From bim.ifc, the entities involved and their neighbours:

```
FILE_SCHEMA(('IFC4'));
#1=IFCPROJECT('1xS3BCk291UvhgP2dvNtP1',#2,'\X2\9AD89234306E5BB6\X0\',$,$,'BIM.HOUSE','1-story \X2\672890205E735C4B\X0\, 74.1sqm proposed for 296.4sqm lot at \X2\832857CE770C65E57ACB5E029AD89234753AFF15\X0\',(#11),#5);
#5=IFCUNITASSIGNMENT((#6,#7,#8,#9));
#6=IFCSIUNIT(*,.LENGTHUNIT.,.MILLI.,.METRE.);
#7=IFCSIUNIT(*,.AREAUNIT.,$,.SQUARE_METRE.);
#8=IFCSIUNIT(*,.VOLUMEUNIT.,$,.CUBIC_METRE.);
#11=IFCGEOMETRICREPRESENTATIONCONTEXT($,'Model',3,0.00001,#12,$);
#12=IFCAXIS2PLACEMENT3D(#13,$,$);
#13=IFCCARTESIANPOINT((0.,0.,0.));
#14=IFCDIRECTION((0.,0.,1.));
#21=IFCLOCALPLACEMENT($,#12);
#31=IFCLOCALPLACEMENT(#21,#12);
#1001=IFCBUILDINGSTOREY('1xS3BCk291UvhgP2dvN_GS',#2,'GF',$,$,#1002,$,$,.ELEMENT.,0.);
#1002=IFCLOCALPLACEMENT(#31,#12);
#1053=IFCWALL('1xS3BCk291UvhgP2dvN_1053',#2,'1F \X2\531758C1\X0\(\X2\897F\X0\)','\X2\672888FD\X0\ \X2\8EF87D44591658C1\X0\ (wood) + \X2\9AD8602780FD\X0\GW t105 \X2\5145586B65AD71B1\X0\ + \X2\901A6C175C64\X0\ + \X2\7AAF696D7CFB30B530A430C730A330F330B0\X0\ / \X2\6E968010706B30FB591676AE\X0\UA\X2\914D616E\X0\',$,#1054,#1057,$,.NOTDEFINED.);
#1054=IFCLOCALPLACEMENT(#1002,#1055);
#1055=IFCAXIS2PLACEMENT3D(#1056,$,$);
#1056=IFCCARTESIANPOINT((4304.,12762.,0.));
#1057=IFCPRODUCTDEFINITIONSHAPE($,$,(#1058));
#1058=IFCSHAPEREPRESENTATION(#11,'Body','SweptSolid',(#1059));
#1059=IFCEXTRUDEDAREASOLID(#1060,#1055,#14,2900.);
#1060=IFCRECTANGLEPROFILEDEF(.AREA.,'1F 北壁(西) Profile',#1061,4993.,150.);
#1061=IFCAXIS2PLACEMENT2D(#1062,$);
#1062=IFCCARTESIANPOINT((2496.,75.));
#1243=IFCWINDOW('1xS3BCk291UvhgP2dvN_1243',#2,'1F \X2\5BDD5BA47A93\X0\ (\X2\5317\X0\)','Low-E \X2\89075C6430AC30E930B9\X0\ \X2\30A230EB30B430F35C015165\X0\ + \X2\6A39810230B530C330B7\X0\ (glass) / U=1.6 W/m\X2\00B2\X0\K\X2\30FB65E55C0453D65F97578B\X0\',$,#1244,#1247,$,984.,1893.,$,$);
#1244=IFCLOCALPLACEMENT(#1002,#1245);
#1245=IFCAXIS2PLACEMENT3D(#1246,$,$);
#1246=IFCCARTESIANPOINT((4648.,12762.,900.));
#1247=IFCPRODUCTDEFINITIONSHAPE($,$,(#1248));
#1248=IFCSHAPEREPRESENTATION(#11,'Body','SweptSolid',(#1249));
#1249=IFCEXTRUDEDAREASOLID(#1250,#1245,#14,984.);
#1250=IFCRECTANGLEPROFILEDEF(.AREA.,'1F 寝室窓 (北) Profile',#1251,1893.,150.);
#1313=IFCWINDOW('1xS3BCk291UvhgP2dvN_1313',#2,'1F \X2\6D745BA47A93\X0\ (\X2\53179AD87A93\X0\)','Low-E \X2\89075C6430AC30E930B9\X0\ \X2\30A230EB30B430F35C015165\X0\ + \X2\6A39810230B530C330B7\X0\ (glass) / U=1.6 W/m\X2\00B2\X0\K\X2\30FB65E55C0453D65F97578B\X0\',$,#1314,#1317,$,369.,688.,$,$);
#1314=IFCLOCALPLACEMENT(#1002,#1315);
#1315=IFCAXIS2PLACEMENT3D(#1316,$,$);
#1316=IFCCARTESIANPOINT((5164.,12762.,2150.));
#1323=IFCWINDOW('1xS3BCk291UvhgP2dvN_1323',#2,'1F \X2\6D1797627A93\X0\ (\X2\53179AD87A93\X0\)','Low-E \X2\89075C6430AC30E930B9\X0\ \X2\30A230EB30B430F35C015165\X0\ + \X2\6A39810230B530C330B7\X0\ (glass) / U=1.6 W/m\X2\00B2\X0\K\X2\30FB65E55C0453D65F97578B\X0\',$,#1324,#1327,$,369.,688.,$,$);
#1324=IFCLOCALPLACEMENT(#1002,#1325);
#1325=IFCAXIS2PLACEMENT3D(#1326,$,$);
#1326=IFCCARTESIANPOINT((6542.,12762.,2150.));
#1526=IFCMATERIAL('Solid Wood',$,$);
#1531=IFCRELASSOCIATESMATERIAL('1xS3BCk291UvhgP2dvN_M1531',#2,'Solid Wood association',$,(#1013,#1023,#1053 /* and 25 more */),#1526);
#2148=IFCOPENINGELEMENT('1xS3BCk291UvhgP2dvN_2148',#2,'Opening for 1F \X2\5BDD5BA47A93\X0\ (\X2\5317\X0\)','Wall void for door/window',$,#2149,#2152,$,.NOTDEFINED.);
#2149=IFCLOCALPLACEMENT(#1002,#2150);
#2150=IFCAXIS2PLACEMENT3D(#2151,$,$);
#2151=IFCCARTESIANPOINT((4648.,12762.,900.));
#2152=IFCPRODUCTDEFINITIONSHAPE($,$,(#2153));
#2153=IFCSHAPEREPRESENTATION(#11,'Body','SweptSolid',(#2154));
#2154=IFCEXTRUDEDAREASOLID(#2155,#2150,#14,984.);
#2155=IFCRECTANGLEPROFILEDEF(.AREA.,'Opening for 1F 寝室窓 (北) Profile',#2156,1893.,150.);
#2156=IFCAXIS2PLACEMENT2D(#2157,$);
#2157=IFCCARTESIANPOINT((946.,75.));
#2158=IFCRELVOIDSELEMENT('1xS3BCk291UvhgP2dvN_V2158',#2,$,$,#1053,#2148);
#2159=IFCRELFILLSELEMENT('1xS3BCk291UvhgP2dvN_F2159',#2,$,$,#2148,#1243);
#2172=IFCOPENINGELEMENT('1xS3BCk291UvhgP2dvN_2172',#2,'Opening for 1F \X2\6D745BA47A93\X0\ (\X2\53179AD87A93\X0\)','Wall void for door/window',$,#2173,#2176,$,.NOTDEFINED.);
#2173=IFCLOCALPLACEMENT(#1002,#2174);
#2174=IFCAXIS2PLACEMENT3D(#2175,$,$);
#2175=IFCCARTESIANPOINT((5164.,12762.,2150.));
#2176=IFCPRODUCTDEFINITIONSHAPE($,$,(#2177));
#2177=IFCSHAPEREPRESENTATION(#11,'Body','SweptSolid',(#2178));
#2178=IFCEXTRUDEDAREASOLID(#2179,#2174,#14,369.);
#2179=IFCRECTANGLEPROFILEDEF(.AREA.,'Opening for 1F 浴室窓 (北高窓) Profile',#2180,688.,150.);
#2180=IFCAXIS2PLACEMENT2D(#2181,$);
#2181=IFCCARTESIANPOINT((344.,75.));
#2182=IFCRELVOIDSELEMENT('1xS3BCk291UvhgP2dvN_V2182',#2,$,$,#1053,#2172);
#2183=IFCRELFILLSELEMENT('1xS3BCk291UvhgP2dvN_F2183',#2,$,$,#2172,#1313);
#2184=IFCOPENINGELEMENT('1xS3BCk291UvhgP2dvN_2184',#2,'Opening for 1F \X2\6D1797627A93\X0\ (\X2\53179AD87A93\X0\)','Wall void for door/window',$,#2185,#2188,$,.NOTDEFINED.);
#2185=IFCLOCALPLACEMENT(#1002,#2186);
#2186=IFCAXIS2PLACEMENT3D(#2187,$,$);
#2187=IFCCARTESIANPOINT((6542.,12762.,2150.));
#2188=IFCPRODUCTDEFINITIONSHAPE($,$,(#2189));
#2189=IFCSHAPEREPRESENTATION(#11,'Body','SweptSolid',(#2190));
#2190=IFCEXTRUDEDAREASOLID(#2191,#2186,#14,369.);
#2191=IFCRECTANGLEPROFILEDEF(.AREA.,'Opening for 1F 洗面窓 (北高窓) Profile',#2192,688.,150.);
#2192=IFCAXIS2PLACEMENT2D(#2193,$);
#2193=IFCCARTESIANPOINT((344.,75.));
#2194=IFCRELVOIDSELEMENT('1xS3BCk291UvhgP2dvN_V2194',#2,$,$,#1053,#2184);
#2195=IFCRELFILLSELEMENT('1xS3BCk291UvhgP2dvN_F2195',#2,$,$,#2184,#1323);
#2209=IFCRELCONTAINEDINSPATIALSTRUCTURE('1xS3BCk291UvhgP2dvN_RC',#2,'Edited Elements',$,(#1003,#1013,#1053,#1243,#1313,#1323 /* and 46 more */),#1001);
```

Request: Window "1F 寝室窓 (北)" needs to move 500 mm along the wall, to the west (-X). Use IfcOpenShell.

```python
import ifcopenshell
import ifcopenshell.api.geometry
import ifcopenshell.util.placement
import ifcopenshell.util.unit

model = ifcopenshell.open("bim.ifc")
unit_scale = ifcopenshell.util.unit.calculate_unit_scale(model)

window = model.by_guid("1xS3BCk291UvhgP2dvN_1243")
opening = window.FillsVoids[0].RelatingOpeningElement
wall = opening.VoidsElements[0].RelatingBuildingElement

wall_matrix = ifcopenshell.util.placement.get_local_placement(wall.ObjectPlacement)
shift = wall_matrix[:3, 0] * -0.5 / unit_scale
before = ifcopenshell.util.placement.get_local_placement(window.ObjectPlacement)[:3, 3].copy()

# The window is not placed relative to its opening, so move both.
for product in (opening, window):
    matrix = ifcopenshell.util.placement.get_local_placement(product.ObjectPlacement)
    matrix[:3, 3] += shift
    ifcopenshell.api.geometry.edit_object_placement(model, product=product, matrix=matrix, is_si=False)

after = ifcopenshell.util.placement.get_local_placement(window.ObjectPlacement)[:3, 3]
print("window moved by", (after - before).round(3) + 0.0)

model.write("bim_rev.ifc")
```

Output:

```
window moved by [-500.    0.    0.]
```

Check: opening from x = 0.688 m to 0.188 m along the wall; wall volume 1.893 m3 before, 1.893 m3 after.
